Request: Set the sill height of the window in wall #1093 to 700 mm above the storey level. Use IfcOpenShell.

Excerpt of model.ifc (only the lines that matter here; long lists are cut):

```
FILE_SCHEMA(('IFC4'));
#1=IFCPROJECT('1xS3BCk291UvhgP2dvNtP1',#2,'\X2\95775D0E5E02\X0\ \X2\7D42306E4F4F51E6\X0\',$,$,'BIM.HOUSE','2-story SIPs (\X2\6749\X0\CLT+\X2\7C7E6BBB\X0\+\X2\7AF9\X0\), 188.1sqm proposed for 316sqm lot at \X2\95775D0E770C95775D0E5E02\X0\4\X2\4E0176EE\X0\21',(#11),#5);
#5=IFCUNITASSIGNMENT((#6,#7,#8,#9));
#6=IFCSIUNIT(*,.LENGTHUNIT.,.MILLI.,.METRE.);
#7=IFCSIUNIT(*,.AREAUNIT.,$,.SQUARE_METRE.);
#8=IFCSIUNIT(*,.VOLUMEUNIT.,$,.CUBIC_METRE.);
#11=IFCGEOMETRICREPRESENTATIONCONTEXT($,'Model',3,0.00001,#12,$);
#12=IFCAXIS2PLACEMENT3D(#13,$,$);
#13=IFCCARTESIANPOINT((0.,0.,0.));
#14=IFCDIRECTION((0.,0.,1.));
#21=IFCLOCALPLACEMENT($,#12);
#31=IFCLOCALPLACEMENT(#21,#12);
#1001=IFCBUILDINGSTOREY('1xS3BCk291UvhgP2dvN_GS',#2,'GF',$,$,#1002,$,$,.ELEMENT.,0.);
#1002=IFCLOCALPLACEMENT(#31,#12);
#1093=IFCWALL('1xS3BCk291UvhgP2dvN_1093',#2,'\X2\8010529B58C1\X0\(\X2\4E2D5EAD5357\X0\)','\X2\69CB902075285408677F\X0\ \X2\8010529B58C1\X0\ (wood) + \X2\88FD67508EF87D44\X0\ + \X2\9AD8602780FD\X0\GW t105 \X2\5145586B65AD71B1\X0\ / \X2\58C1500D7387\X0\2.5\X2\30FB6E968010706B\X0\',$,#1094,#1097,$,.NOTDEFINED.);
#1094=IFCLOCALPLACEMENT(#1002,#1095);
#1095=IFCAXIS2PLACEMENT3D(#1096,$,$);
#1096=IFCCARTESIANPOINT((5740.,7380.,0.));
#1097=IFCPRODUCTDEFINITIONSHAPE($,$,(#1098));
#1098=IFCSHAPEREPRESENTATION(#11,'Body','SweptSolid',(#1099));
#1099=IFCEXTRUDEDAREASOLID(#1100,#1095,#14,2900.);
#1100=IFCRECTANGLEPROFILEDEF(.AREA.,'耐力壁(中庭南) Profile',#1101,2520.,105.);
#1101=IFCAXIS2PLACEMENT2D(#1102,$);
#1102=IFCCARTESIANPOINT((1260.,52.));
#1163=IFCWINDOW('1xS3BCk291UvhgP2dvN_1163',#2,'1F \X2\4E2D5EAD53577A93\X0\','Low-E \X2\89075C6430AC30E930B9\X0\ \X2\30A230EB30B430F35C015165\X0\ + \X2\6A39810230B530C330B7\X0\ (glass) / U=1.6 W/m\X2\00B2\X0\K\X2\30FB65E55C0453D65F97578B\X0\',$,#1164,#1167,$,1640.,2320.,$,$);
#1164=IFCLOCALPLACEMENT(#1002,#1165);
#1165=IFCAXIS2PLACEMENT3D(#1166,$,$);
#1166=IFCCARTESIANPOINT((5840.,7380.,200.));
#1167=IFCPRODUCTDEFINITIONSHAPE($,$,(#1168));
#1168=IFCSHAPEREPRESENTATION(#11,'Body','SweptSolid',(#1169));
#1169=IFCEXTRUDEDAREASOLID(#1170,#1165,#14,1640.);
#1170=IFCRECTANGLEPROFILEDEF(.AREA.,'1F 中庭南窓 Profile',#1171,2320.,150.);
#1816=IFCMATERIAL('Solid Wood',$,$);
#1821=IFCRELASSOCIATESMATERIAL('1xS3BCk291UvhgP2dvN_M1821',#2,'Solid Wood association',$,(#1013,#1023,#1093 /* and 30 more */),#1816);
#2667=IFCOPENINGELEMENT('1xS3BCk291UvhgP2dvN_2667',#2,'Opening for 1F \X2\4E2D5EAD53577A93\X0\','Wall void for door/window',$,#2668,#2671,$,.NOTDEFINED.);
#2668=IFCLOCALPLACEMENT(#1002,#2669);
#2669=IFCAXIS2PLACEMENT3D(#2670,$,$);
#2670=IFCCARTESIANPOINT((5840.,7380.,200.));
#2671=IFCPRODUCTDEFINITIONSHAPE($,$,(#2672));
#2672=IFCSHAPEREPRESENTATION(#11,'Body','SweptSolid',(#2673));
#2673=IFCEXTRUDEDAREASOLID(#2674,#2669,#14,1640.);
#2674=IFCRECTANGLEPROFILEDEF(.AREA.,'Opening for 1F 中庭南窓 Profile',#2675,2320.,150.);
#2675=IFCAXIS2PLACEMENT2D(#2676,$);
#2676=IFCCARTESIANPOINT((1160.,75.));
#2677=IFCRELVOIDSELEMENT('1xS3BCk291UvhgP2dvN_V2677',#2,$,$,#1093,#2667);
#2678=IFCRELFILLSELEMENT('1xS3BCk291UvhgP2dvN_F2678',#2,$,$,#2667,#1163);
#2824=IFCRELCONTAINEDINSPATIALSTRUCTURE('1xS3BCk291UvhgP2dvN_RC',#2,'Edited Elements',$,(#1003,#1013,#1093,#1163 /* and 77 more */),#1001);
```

```python
import numpy as np
import ifcopenshell
import ifcopenshell.api.geometry
import ifcopenshell.geom
import ifcopenshell.util.element
import ifcopenshell.util.placement
import ifcopenshell.util.shape
import ifcopenshell.util.unit

model = ifcopenshell.open("model.ifc")
unit_scale = ifcopenshell.util.unit.calculate_unit_scale(model)

window = model.by_guid("1xS3BCk291UvhgP2dvN_1163")
opening = window.FillsVoids[0].RelatingOpeningElement
storey = ifcopenshell.util.element.get_container(window, ifc_class="IfcBuildingStorey")
level = ifcopenshell.util.placement.get_local_placement(storey.ObjectPlacement)[2, 3]

# The opening's origin need not be at the sill, so measure its lowest point.
shape = ifcopenshell.geom.create_shape(ifcopenshell.geom.settings(), opening)
bottom = ifcopenshell.util.shape.get_shape_bottom_elevation(shape, shape.geometry) / unit_scale
dz = level + 700.0 - bottom

shift = np.array([0.0, 0.0, dz])
# The window is not placed relative to its opening, so move both.
for product in (opening, window):
    matrix = ifcopenshell.util.placement.get_local_placement(product.ObjectPlacement)
    matrix[:3, 3] += shift
    ifcopenshell.api.geometry.edit_object_placement(model, product=product, matrix=matrix, is_si=False)

print(f"moved by {dz * unit_scale:+.3f} m")

model.write("model_updated.ifc")
```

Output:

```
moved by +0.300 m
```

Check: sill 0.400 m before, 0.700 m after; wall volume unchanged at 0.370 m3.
